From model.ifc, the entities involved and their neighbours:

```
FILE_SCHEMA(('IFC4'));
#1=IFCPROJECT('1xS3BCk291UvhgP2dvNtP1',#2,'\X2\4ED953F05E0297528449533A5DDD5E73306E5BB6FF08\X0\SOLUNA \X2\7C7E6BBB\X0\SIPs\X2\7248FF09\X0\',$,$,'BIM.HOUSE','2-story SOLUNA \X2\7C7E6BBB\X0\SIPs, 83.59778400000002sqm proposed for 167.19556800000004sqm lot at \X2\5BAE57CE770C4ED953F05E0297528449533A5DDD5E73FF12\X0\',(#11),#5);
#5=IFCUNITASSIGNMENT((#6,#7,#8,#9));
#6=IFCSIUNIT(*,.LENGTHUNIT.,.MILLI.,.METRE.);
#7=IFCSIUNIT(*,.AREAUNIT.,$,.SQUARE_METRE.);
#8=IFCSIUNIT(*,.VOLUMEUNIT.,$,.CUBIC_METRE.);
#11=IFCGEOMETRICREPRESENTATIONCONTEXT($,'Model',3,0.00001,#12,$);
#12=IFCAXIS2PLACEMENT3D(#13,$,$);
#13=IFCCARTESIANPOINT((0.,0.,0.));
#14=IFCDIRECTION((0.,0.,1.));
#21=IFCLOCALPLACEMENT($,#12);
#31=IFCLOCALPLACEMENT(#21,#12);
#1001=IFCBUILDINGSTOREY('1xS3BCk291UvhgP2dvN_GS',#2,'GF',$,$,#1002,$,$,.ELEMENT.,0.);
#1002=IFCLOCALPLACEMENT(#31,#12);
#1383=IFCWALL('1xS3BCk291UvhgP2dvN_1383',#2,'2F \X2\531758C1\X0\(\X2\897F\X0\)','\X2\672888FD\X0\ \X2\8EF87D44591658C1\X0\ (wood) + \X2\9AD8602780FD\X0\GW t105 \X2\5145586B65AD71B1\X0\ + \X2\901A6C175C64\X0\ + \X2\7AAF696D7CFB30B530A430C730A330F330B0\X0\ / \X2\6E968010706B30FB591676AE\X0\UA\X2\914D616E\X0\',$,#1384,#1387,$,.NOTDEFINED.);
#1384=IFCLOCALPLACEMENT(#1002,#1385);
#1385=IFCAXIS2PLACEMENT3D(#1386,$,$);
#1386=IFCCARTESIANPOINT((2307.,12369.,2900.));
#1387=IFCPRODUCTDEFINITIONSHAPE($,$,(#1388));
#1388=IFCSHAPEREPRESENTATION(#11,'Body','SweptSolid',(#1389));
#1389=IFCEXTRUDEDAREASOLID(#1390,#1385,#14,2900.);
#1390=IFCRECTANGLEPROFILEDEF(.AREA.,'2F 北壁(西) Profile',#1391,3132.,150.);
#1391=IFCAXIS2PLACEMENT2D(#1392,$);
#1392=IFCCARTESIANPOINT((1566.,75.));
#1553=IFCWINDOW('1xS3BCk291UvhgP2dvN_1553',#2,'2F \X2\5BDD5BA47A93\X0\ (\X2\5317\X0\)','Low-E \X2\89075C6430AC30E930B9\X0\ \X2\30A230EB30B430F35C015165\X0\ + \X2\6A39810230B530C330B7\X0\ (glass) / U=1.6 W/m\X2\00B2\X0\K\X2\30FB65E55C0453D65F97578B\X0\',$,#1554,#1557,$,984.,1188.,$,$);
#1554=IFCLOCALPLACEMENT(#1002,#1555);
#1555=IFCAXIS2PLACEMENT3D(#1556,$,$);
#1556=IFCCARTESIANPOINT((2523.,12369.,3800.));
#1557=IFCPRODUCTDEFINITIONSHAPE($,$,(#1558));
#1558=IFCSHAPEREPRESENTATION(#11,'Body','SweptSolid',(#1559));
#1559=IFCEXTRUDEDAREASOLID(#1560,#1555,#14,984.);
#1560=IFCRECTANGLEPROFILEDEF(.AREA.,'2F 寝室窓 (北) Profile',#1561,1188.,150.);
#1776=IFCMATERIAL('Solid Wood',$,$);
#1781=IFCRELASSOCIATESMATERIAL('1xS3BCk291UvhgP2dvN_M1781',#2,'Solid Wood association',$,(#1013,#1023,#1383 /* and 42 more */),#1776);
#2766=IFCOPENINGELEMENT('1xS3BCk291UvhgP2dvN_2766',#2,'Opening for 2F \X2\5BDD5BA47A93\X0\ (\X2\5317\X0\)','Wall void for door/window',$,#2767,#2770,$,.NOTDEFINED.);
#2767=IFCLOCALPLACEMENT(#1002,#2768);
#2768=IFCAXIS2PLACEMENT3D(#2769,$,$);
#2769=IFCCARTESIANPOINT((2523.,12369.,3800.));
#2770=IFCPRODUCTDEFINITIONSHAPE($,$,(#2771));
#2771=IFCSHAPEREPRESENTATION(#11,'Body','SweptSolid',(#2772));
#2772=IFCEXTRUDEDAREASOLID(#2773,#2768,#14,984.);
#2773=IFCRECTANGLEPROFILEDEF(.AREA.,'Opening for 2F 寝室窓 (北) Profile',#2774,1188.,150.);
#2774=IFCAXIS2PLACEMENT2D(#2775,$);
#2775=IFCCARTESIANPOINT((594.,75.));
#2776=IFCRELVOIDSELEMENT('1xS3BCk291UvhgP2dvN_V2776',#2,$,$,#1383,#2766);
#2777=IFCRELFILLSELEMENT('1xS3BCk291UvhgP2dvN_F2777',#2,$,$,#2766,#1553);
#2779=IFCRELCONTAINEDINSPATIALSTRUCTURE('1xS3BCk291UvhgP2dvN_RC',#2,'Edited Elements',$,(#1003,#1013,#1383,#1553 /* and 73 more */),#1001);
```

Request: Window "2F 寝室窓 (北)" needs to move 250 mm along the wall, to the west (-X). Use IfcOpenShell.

```python
import ifcopenshell
import ifcopenshell.api.geometry
import ifcopenshell.util.placement

model = ifcopenshell.open("model.ifc")

window = model.by_guid("1xS3BCk291UvhgP2dvN_1553")
opening = window.FillsVoids[0].RelatingOpeningElement
wall = opening.VoidsElements[0].RelatingBuildingElement

wall_matrix = ifcopenshell.util.placement.get_local_placement(wall.ObjectPlacement)
shift = wall_matrix[:3, 0] * -250.0
before = ifcopenshell.util.placement.get_local_placement(window.ObjectPlacement)[:3, 3].copy()

# The window is not placed relative to its opening, so move both.
for product in (opening, window):
    matrix = ifcopenshell.util.placement.get_local_placement(product.ObjectPlacement)
    matrix[:3, 3] += shift
    ifcopenshell.api.geometry.edit_object_placement(model, product=product, matrix=matrix, is_si=False)

after = ifcopenshell.util.placement.get_local_placement(window.ObjectPlacement)[:3, 3]
print("window moved by", (after - before).round(3) + 0.0)

model.write("model_updated.ifc")
```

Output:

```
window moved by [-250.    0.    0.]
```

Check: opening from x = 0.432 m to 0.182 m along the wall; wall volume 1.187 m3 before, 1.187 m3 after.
